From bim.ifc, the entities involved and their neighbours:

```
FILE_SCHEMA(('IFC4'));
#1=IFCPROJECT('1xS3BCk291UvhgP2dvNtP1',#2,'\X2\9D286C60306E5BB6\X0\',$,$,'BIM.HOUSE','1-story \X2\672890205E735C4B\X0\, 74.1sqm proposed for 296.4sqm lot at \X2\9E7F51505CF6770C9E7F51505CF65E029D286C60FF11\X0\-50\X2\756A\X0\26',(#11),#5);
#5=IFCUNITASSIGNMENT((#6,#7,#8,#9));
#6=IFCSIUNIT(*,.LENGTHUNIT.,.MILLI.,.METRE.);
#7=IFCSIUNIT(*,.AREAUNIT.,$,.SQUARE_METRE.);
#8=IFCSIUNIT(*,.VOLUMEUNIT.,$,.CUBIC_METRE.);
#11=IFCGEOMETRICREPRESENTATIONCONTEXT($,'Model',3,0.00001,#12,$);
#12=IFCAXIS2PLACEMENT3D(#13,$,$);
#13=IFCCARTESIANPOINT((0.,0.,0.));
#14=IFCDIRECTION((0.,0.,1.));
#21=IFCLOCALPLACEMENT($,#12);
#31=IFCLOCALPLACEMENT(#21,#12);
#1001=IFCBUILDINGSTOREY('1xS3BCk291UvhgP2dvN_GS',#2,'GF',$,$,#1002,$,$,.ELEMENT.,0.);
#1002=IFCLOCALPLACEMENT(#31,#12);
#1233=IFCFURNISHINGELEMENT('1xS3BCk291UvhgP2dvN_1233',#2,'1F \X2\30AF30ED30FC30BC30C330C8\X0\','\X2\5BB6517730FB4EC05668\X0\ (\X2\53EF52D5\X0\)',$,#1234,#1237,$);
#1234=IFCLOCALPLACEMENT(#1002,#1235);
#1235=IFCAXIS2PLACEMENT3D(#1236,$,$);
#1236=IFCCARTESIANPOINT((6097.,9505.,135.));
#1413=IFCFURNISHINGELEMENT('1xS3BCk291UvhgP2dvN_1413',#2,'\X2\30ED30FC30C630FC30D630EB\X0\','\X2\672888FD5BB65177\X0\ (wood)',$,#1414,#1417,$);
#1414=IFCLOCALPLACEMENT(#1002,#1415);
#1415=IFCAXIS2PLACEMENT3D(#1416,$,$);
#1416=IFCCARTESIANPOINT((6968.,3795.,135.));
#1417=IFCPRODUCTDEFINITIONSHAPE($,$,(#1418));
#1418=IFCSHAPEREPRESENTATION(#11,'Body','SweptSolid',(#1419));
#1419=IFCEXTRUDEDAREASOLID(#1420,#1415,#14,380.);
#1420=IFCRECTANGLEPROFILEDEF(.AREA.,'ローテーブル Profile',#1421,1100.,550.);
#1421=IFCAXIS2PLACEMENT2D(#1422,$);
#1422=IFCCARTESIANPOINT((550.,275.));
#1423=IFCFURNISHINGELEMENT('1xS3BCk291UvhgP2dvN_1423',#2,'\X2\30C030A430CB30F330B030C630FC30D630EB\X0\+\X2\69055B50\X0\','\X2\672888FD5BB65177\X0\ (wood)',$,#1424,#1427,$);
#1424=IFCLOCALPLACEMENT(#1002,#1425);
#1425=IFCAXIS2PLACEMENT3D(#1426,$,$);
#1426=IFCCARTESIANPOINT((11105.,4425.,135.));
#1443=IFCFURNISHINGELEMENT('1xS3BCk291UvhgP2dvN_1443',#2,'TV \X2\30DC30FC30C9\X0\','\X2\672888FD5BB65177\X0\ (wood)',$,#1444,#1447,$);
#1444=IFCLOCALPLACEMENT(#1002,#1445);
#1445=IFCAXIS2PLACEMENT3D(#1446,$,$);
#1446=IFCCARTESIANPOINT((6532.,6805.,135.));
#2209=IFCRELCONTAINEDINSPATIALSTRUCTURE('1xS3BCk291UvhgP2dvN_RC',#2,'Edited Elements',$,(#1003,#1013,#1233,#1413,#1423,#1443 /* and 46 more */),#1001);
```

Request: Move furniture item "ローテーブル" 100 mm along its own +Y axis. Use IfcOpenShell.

```python
import ifcopenshell
import ifcopenshell.api.geometry
import ifcopenshell.util.placement
import ifcopenshell.util.unit

model = ifcopenshell.open("bim.ifc")
unit_scale = ifcopenshell.util.unit.calculate_unit_scale(model)

item = model.by_guid("1xS3BCk291UvhgP2dvN_1413")
matrix = ifcopenshell.util.placement.get_local_placement(item.ObjectPlacement)
matrix[:3, 3] += matrix[:3, 1] * 0.1 / unit_scale
ifcopenshell.api.geometry.edit_object_placement(model, product=item, matrix=matrix, is_si=False)

print(ifcopenshell.util.placement.get_local_placement(item.ObjectPlacement).round(3) + 0.0)

model.write("bim_rev.ifc")
```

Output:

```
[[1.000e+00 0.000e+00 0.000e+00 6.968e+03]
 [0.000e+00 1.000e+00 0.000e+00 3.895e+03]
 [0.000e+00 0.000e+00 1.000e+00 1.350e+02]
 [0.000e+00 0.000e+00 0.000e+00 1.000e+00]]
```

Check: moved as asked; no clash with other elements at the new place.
